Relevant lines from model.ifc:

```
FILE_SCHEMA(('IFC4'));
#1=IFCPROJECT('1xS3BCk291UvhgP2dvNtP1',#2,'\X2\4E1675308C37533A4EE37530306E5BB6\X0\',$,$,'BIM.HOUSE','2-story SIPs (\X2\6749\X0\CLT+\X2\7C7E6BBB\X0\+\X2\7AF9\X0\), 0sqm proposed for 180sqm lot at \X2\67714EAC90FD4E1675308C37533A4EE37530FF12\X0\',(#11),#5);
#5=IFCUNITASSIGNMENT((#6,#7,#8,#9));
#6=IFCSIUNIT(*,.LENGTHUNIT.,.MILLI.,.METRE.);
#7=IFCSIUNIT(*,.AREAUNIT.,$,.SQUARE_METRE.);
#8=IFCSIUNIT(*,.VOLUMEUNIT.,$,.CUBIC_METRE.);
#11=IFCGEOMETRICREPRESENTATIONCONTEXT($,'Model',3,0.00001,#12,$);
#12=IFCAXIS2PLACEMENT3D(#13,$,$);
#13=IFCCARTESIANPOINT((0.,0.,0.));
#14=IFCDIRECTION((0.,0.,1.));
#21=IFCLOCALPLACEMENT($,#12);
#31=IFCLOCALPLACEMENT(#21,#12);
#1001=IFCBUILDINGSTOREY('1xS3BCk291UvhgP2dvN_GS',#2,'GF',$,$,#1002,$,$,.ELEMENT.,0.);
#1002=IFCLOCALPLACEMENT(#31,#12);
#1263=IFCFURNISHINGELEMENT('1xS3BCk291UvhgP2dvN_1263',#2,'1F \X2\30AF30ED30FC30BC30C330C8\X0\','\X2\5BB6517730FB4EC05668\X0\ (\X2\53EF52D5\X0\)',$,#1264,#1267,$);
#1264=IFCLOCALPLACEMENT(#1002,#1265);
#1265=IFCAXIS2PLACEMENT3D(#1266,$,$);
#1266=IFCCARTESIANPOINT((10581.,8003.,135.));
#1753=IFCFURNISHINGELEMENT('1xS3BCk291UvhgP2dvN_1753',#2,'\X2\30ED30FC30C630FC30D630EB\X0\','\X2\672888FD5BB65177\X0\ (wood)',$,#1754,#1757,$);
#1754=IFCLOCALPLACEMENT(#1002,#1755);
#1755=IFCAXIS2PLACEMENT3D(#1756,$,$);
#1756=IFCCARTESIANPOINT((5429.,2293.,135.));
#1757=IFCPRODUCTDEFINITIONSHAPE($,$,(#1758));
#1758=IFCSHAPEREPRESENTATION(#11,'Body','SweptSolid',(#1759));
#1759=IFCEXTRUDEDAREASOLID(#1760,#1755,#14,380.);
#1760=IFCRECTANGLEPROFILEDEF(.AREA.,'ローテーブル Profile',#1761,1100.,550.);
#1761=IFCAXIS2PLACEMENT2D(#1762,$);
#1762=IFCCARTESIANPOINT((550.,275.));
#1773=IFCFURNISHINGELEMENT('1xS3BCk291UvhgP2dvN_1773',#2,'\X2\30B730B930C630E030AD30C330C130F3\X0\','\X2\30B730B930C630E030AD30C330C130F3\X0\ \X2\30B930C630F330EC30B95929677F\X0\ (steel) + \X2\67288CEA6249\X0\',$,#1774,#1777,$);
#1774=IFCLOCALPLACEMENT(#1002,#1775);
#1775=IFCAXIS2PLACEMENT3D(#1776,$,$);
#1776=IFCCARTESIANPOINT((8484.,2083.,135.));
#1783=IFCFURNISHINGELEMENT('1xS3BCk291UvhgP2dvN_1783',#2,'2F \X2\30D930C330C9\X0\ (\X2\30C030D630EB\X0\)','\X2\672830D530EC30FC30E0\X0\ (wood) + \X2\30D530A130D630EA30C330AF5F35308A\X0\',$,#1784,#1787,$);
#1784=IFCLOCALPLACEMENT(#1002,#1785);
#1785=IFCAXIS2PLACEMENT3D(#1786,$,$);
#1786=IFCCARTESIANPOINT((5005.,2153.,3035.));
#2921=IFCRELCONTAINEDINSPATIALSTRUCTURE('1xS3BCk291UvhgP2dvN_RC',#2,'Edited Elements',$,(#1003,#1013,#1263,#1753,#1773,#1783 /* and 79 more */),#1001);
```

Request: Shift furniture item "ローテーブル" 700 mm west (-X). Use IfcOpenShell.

```python
import ifcopenshell
import ifcopenshell.api.geometry
import ifcopenshell.util.placement
import ifcopenshell.util.unit

model = ifcopenshell.open("model.ifc")
unit_scale = ifcopenshell.util.unit.calculate_unit_scale(model)

item = model.by_id(1753)
matrix = ifcopenshell.util.placement.get_local_placement(item.ObjectPlacement)
matrix[0, 3] -= 0.7 / unit_scale
ifcopenshell.api.geometry.edit_object_placement(model, product=item, matrix=matrix, is_si=False)

print(ifcopenshell.util.placement.get_local_placement(item.ObjectPlacement).round(3) + 0.0)

model.write("model_v2.ifc")
```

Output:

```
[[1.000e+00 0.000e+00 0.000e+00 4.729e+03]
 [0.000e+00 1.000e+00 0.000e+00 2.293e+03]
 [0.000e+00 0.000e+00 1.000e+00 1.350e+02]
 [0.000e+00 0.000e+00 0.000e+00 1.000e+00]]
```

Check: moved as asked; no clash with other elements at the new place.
